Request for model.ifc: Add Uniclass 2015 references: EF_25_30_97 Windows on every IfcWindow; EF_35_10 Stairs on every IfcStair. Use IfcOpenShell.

First a look at what the model holds.

```python
import ifcopenshell

model = ifcopenshell.open("model.ifc")
print(model.schema)
print("classifications:", [c.Name for c in model.by_type("IfcClassification")])
for ifc_class in ("IfcDoor", "IfcRoof", "IfcStair", "IfcWall", "IfcWindow"):
    print(ifc_class, len(model.by_type(ifc_class)))
```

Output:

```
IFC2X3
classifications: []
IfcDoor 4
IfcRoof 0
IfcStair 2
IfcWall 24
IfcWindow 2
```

```python
import ifcopenshell
import ifcopenshell.api.classification

model = ifcopenshell.open("model.ifc")

# IFC2X3 requires Source and Edition and has no link from the project to the system.
system = model.create_entity("IfcClassification", Source="NBS", Edition="2015", Name="Uniclass 2015")

codes = {
    "IfcWindow": ("EF_25_30_97", "Windows"),
    "IfcStair": ("EF_35_10", "Stairs"),
}
for ifc_class, (code, name) in codes.items():
    products = model.by_type(ifc_class)
    ifcopenshell.api.classification.add_reference(
        model, products=products, classification=system, identification=code, name=name
    )
    print(code, len(products))

model.write("model_rev.ifc")
```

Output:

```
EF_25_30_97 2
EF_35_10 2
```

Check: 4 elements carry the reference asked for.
